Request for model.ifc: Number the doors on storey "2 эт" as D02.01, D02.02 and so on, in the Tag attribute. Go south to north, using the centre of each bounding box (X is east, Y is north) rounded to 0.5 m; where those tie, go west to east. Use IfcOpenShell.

First a look at what the model holds.

```python
import ifcopenshell
import ifcopenshell.util.element
import ifcopenshell.util.placement

model = ifcopenshell.open("model.ifc")
print(model.schema)
storey = next(s for s in model.by_type("IfcBuildingStorey") if s.Name == "2 эт")
doors = [e for e in ifcopenshell.util.element.get_decomposition(storey) if e.is_a("IfcDoor")]
for e in sorted(doors, key=lambda e: e.id()):
    origin = ifcopenshell.util.placement.get_local_placement(e.ObjectPlacement)[:3, 3]
    print(e.id(), e.Tag, e.Name, origin.round(2) + 0.0, sep=" | ")
```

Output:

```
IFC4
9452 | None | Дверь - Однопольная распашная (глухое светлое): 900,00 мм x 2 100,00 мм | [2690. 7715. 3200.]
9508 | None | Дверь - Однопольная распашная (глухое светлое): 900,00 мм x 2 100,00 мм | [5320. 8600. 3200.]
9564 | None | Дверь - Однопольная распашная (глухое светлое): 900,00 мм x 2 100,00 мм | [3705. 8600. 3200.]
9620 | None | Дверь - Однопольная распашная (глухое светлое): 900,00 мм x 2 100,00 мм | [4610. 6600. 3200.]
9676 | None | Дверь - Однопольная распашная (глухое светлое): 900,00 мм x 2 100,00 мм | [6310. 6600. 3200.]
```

```python
import ifcopenshell
import ifcopenshell.geom
import ifcopenshell.util.element
import ifcopenshell.util.shape

model = ifcopenshell.open("model.ifc")
settings = ifcopenshell.geom.settings()
settings.set("use-world-coords", True)


def centre(element):
    shape = ifcopenshell.geom.create_shape(settings, element)
    return ifcopenshell.util.shape.get_bbox_centroid(shape.geometry)


storey = next(s for s in model.by_type("IfcBuildingStorey") if s.Name == "2 эт")
doors = [e for e in ifcopenshell.util.element.get_decomposition(storey) if e.is_a("IfcDoor")]

# Insertion points can sit at a corner or the storey origin, so sort by the geometry (in metres).
centres = {e: centre(e) for e in doors}
doors.sort(key=lambda e: (round(centres[e][1] / 0.5), centres[e][0]))

for i, e in enumerate(doors, start=1):
    number = f"D02.{i:02d}"
    e.Tag = number
    print(e.id(), number)

model.write("model-out.ifc")
```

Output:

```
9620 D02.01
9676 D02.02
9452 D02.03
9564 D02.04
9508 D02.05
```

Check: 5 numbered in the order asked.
